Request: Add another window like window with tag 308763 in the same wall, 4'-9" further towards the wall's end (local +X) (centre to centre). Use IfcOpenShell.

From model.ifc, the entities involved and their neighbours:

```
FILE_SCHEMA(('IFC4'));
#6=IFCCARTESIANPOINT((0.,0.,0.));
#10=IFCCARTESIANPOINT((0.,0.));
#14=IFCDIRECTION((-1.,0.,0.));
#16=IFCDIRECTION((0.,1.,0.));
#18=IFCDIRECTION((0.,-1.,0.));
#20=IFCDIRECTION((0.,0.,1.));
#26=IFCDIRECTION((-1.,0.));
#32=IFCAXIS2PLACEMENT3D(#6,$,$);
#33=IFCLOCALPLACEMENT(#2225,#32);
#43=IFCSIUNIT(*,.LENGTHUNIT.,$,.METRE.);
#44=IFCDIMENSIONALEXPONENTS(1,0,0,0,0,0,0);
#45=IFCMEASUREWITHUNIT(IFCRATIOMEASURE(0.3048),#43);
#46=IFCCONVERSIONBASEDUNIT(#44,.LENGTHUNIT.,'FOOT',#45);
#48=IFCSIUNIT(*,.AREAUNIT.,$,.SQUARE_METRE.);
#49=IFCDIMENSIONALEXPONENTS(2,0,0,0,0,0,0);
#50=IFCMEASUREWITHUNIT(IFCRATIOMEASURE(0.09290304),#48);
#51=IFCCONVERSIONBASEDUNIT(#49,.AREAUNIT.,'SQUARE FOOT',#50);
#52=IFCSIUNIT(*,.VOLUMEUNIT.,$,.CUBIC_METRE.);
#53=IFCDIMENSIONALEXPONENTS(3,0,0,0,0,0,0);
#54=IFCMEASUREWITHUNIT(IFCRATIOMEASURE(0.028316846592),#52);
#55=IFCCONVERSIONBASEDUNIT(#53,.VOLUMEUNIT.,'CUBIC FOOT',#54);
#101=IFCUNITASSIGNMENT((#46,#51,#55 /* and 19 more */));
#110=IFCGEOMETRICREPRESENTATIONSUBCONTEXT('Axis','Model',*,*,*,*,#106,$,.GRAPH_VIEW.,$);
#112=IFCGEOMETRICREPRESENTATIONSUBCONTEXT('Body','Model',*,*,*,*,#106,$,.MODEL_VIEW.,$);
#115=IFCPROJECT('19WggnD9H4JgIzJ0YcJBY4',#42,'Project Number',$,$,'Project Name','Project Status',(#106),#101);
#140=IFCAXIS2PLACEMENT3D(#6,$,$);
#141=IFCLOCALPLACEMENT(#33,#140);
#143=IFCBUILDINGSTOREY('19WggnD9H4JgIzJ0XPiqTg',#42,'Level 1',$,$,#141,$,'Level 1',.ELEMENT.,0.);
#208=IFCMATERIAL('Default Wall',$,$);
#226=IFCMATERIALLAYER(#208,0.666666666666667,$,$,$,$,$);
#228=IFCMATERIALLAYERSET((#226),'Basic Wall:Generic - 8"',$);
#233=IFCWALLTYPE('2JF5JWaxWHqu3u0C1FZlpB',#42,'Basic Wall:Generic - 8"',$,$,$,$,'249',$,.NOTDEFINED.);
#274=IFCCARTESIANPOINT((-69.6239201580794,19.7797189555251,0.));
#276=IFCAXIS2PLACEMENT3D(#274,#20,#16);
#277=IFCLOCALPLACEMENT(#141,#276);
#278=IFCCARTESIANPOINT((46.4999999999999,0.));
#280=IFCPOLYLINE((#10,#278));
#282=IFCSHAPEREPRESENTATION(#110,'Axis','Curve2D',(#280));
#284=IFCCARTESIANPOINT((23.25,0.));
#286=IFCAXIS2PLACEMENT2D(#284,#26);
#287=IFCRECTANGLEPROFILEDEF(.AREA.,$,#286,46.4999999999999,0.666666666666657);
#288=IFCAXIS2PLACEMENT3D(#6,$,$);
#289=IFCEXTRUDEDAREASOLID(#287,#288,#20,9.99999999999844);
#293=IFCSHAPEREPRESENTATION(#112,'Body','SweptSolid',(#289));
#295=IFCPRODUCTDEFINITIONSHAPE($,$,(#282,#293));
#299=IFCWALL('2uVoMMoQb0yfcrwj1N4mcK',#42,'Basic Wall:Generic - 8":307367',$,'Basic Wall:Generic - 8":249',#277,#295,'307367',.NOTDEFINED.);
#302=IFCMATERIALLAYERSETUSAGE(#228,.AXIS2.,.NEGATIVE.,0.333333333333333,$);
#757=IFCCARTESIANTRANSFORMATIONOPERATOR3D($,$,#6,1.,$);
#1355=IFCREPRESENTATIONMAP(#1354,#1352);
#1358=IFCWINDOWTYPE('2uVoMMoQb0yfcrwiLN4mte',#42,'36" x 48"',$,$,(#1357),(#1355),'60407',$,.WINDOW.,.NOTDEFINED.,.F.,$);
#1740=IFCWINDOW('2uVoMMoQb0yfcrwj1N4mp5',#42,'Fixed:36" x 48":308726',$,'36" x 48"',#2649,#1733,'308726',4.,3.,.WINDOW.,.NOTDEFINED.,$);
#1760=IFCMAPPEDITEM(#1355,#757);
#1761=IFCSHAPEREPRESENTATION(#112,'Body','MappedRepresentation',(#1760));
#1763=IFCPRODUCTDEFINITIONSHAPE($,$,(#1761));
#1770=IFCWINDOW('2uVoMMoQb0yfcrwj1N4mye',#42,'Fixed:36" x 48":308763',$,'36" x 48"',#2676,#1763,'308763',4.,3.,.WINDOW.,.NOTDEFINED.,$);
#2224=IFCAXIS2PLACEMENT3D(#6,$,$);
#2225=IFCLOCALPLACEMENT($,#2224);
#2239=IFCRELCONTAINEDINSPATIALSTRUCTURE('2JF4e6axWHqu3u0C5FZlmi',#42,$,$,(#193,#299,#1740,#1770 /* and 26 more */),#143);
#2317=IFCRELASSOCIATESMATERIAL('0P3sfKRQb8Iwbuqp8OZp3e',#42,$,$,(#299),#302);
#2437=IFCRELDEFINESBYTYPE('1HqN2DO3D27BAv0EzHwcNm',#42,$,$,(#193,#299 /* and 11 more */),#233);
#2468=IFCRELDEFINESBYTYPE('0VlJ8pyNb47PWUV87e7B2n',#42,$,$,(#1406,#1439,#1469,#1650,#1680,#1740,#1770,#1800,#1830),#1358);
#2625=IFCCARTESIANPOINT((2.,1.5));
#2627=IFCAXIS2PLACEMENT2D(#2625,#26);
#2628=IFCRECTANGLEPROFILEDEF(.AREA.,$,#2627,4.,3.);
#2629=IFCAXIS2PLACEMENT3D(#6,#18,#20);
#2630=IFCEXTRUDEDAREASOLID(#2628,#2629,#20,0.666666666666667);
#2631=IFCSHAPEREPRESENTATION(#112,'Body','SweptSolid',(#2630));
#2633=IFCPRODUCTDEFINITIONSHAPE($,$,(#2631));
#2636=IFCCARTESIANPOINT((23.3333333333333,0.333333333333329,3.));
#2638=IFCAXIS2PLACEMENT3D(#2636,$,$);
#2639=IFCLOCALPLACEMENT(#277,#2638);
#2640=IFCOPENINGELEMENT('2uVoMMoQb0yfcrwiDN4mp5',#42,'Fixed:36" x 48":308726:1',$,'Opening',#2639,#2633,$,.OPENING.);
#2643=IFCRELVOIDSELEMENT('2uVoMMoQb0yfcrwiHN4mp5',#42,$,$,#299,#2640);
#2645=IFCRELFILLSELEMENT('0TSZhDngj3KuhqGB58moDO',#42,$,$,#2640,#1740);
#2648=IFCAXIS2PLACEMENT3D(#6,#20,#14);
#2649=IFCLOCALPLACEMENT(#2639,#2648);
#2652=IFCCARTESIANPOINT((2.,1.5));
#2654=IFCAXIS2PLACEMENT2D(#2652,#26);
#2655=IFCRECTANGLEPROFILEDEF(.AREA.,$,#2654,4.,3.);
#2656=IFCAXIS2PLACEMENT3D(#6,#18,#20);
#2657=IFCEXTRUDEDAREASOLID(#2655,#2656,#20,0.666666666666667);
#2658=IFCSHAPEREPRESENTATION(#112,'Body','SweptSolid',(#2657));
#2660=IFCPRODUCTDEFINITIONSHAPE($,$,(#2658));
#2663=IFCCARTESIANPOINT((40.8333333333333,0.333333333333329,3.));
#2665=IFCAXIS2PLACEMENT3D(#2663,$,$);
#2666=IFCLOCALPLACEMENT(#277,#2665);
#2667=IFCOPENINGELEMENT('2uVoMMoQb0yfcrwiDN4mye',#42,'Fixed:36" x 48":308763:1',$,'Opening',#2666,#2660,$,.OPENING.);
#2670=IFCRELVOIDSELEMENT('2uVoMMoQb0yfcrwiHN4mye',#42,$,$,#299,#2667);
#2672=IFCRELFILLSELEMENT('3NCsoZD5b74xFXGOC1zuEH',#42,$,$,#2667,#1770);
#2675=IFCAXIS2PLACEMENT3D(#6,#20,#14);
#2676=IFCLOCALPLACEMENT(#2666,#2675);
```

```python
import ifcopenshell
import ifcopenshell.api.feature
import ifcopenshell.api.geometry
import ifcopenshell.api.root
import ifcopenshell.geom
import ifcopenshell.util.element
import ifcopenshell.util.placement
import ifcopenshell.util.shape
import ifcopenshell.util.unit

model = ifcopenshell.open("model.ifc")
unit_scale = ifcopenshell.util.unit.calculate_unit_scale(model)
settings = ifcopenshell.geom.settings()


def volume(element):
    """Net volume in cubic metres, openings subtracted."""
    shape = ifcopenshell.geom.create_shape(settings, element)
    return ifcopenshell.util.shape.get_volume(shape.geometry)


def reuse_history(source, copy):
    """copy_class also copies each property set's owner history, people and application; keep the originals."""
    for rel in copy.IsDefinedBy:
        if rel.is_a("IfcRelDefinesByProperties") and (history := rel.RelatingPropertyDefinition.OwnerHistory):
            rel.RelatingPropertyDefinition.OwnerHistory = source.OwnerHistory
            ifcopenshell.util.element.remove_deep2(model, history)


window = model.by_id(1770)
opening = window.FillsVoids[0].RelatingOpeningElement
wall = opening.VoidsElements[0].RelatingBuildingElement
before = volume(wall)
shift = ifcopenshell.util.placement.get_local_placement(wall.ObjectPlacement)[:3, 0] * 57 * 0.0254 / unit_scale

# copy_class copies the void relationship, type, container and properties, but no geometry.
new_opening = ifcopenshell.api.root.copy_class(model, product=opening)
new_opening.Representation = ifcopenshell.util.element.copy_deep(
    model, opening.Representation, exclude=["IfcGeometricRepresentationContext", "IfcRepresentationMap"]
)
new_opening.Name = 'Fixed:36" x 48"'
new_window = ifcopenshell.api.root.copy_class(model, product=window)
new_window.Representation = ifcopenshell.util.element.copy_deep(
    model, window.Representation, exclude=["IfcGeometricRepresentationContext", "IfcRepresentationMap"]
)
new_window.Name = 'Fixed:36" x 48"'
new_window.Tag = None
reuse_history(window, new_window)
ifcopenshell.api.feature.add_filling(model, opening=new_opening, element=new_window)

for old, new in ((opening, new_opening), (window, new_window)):
    matrix = ifcopenshell.util.placement.get_local_placement(old.ObjectPlacement)
    matrix[:3, 3] += shift
    ifcopenshell.api.geometry.edit_object_placement(model, product=new, matrix=matrix, is_si=False)

after = volume(wall)

print(f"wall volume {before:.3f} -> {after:.3f} m3")

model.write("model_v2.ifc")
```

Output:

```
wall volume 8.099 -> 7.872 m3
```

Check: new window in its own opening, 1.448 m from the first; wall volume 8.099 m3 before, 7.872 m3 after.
